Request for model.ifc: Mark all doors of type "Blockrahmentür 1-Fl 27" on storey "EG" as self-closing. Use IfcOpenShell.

First a look at what the model holds.

```python
import ifcopenshell
import ifcopenshell.util.element

model = ifcopenshell.open("model.ifc")
print(model.schema)
storey = next(s for s in model.by_type("IfcBuildingStorey") if s.Name == "EG")
doors = [e for e in ifcopenshell.util.element.get_decomposition(storey) if e.is_a("IfcDoor")]
seen = {}
for e in doors:
    element_type = ifcopenshell.util.element.get_type(e)
    key = (element_type.Name if element_type != e and element_type else None, ifcopenshell.util.element.get_pset(e, "Pset_DoorCommon", "SelfClosing"))
    seen[key] = seen.get(key, 0) + 1
for (name, value), count in sorted(seen.items(), key=str):
    print(count, "x", name, "|", value)
```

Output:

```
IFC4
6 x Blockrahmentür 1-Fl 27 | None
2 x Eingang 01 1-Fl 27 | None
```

```python
import ifcopenshell
import ifcopenshell.api.pset
import ifcopenshell.util.element

model = ifcopenshell.open("model.ifc")

storey = next(s for s in model.by_type("IfcBuildingStorey") if s.Name == "EG")
doors = [e for e in ifcopenshell.util.element.get_decomposition(storey) if e.is_a("IfcDoor")]

count = 0
for e in doors:
    element_type = ifcopenshell.util.element.get_type(e)
    if element_type in (None, e) or element_type.Name != "Blockrahmentür 1-Fl 27":
        continue
    # add_pset returns the element's existing set when there is one.
    pset = ifcopenshell.api.pset.add_pset(model, product=e, name="Pset_DoorCommon")
    ifcopenshell.api.pset.edit_pset(model, pset=pset, properties={"SelfClosing": True})
    count += 1

print(count, "doors updated")

model.write("model_rev.ifc")
```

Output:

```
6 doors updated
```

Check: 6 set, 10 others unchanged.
